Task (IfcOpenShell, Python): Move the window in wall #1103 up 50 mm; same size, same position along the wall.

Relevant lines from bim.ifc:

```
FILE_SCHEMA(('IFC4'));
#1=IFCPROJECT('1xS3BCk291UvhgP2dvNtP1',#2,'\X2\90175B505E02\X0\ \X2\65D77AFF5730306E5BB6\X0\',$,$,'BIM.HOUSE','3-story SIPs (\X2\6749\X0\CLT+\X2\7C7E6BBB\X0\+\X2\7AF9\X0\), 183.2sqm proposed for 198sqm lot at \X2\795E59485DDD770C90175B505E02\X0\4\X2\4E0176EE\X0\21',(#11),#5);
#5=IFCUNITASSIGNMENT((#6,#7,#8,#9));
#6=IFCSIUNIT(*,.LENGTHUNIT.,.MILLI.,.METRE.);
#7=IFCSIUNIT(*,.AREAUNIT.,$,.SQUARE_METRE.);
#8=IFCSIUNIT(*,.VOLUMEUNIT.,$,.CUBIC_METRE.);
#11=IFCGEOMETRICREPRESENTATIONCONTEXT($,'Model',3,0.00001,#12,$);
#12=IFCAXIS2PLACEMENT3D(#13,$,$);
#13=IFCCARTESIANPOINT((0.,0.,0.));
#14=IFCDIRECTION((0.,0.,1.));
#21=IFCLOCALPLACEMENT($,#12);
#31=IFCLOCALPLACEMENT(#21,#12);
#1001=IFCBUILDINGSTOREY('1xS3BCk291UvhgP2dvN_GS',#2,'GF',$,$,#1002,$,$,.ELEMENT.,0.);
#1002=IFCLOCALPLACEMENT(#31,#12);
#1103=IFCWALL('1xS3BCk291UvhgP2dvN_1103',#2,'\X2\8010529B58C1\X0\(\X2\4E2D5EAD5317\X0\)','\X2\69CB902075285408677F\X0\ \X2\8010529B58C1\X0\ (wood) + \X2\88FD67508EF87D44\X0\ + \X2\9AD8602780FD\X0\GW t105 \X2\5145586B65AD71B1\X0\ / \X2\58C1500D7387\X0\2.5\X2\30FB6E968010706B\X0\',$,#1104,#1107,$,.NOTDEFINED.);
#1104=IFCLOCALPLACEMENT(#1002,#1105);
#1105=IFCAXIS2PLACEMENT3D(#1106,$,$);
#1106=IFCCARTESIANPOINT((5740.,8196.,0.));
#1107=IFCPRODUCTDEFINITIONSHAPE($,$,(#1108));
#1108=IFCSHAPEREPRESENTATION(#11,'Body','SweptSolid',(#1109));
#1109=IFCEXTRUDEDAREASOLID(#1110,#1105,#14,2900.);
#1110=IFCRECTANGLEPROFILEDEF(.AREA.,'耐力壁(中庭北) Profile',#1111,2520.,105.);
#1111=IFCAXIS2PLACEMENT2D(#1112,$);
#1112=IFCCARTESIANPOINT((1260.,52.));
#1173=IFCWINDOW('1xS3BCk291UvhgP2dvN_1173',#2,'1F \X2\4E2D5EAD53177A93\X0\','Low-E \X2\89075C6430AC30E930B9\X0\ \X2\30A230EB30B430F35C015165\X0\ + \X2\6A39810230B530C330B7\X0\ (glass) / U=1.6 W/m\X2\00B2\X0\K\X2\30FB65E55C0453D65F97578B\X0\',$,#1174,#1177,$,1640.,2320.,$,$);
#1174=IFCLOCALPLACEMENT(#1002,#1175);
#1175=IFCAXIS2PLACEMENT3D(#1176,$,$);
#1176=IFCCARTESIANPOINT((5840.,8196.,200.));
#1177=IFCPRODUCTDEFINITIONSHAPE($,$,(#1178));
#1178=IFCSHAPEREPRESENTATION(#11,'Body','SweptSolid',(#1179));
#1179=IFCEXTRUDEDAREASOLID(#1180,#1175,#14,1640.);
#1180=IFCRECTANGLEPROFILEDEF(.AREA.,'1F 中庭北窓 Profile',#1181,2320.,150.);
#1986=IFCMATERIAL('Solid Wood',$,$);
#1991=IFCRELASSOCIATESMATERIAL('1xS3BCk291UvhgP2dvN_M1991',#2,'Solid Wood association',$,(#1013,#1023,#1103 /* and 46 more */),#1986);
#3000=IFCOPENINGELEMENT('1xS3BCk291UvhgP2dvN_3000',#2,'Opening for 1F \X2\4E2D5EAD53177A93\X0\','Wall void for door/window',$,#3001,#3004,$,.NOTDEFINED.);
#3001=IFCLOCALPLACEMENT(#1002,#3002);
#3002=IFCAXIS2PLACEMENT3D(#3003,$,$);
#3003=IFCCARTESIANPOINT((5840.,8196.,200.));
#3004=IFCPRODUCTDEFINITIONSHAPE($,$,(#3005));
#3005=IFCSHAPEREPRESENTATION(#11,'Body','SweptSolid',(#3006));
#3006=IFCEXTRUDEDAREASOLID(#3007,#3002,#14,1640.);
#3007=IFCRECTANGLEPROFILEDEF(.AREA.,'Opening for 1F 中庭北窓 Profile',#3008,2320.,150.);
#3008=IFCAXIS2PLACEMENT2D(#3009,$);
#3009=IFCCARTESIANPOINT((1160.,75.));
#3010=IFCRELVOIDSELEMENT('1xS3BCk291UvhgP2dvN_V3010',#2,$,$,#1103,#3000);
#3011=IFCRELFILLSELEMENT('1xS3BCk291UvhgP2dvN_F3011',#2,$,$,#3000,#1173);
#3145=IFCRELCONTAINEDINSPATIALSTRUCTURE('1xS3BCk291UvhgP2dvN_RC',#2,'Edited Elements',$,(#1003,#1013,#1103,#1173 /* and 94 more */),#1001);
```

```python
import numpy as np
import ifcopenshell
import ifcopenshell.api.geometry
import ifcopenshell.util.placement
import ifcopenshell.util.unit

model = ifcopenshell.open("bim.ifc")
unit_scale = ifcopenshell.util.unit.calculate_unit_scale(model)

window = model.by_id(1173)
opening = window.FillsVoids[0].RelatingOpeningElement
dz = 50.0

shift = np.array([0.0, 0.0, dz])
# The window is not placed relative to its opening, so move both.
for product in (opening, window):
    matrix = ifcopenshell.util.placement.get_local_placement(product.ObjectPlacement)
    matrix[:3, 3] += shift
    ifcopenshell.api.geometry.edit_object_placement(model, product=product, matrix=matrix, is_si=False)

print(f"moved by {dz * unit_scale:+.3f} m")

model.write("bim_updated.ifc")
```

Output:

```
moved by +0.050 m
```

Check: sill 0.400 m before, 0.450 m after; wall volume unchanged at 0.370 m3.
